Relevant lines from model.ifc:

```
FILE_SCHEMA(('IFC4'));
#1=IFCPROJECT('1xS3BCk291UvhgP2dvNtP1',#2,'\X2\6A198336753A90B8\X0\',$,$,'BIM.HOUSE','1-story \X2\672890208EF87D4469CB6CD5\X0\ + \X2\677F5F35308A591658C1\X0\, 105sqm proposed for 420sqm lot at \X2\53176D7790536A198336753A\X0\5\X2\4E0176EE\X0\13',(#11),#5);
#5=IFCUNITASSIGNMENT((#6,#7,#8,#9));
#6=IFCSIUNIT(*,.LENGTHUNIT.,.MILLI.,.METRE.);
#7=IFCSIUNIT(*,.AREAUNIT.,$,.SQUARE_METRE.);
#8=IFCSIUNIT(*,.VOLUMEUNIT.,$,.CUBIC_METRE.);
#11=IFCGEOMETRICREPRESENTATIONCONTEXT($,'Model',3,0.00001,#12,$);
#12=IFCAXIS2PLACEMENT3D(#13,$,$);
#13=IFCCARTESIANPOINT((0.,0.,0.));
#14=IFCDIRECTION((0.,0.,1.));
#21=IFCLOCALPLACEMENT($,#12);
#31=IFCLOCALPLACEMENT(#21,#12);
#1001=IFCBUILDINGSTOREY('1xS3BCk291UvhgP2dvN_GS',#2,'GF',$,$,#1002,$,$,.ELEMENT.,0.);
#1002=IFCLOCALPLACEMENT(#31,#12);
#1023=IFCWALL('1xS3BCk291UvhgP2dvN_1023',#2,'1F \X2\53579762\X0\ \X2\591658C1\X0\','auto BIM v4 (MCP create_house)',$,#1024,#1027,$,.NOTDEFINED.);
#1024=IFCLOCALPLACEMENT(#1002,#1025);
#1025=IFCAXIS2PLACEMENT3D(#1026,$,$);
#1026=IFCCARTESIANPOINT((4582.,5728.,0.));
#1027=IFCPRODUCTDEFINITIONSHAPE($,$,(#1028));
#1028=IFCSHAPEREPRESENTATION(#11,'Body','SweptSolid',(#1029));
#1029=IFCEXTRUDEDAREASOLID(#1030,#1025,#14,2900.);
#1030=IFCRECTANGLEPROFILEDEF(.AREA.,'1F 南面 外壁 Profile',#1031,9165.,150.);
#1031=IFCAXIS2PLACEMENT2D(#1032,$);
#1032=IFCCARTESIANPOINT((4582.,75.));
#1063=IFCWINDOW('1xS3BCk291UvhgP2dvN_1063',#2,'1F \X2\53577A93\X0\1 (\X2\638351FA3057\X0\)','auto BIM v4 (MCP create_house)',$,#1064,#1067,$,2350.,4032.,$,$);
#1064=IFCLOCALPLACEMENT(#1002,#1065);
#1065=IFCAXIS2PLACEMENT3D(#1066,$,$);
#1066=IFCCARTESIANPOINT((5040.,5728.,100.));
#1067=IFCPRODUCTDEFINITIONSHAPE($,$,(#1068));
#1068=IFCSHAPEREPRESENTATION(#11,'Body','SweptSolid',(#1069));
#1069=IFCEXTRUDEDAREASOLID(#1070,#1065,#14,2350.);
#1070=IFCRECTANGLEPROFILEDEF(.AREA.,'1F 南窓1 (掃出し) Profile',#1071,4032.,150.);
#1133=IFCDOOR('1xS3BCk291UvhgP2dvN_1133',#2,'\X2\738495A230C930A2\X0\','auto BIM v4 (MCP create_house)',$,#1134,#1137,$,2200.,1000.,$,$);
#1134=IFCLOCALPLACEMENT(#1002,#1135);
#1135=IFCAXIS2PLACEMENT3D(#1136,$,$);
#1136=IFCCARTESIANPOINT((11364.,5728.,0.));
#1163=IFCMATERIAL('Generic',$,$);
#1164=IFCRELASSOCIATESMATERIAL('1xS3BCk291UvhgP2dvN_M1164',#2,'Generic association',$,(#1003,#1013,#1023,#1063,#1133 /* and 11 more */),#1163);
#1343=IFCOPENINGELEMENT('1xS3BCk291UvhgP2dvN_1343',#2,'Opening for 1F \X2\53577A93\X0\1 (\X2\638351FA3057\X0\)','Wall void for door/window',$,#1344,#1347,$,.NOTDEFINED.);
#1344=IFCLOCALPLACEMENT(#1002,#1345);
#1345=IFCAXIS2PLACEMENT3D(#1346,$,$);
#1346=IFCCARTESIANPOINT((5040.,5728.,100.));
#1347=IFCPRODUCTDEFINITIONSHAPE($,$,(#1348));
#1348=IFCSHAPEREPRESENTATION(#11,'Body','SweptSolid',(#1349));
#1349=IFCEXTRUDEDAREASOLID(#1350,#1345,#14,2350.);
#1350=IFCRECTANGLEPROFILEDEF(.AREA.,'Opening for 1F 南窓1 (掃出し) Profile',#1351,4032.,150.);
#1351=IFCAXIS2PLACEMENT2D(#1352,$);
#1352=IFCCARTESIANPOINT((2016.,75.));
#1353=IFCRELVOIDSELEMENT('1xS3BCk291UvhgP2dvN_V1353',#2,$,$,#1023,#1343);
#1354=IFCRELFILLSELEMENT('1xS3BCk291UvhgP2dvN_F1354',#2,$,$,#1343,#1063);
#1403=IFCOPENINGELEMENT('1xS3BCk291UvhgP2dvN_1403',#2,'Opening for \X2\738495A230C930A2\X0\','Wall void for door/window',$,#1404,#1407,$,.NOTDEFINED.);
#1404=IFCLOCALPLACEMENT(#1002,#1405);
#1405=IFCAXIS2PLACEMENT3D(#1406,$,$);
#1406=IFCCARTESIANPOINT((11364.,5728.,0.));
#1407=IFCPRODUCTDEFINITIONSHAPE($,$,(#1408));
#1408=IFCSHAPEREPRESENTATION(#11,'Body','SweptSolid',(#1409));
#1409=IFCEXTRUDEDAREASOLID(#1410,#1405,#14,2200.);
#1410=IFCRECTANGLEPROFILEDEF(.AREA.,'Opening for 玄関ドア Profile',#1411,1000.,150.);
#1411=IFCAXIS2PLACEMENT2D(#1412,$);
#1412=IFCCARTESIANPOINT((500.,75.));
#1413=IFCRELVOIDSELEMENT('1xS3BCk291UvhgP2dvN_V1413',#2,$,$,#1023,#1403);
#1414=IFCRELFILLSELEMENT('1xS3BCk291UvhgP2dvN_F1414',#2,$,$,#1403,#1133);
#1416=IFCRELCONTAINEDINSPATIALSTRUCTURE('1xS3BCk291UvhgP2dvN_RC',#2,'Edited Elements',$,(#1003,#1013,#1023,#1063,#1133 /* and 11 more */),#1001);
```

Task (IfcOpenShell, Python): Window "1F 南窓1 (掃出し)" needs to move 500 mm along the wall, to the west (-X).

```python
import ifcopenshell
import ifcopenshell.api.geometry
import ifcopenshell.util.placement
import ifcopenshell.util.unit

model = ifcopenshell.open("model.ifc")
unit_scale = ifcopenshell.util.unit.calculate_unit_scale(model)

window = model.by_guid("1xS3BCk291UvhgP2dvN_1063")
opening = window.FillsVoids[0].RelatingOpeningElement
wall = opening.VoidsElements[0].RelatingBuildingElement

wall_matrix = ifcopenshell.util.placement.get_local_placement(wall.ObjectPlacement)
shift = wall_matrix[:3, 0] * -0.5 / unit_scale
before = ifcopenshell.util.placement.get_local_placement(window.ObjectPlacement)[:3, 3].copy()

# The window is not placed relative to its opening, so move both.
for product in (opening, window):
    matrix = ifcopenshell.util.placement.get_local_placement(product.ObjectPlacement)
    matrix[:3, 3] += shift
    ifcopenshell.api.geometry.edit_object_placement(model, product=product, matrix=matrix, is_si=False)

after = ifcopenshell.util.placement.get_local_placement(window.ObjectPlacement)[:3, 3]
print("window moved by", (after - before).round(3) + 0.0)

model.write("model_updated.ifc")
```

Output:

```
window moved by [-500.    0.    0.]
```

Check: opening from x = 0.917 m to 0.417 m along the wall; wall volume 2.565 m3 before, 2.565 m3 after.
